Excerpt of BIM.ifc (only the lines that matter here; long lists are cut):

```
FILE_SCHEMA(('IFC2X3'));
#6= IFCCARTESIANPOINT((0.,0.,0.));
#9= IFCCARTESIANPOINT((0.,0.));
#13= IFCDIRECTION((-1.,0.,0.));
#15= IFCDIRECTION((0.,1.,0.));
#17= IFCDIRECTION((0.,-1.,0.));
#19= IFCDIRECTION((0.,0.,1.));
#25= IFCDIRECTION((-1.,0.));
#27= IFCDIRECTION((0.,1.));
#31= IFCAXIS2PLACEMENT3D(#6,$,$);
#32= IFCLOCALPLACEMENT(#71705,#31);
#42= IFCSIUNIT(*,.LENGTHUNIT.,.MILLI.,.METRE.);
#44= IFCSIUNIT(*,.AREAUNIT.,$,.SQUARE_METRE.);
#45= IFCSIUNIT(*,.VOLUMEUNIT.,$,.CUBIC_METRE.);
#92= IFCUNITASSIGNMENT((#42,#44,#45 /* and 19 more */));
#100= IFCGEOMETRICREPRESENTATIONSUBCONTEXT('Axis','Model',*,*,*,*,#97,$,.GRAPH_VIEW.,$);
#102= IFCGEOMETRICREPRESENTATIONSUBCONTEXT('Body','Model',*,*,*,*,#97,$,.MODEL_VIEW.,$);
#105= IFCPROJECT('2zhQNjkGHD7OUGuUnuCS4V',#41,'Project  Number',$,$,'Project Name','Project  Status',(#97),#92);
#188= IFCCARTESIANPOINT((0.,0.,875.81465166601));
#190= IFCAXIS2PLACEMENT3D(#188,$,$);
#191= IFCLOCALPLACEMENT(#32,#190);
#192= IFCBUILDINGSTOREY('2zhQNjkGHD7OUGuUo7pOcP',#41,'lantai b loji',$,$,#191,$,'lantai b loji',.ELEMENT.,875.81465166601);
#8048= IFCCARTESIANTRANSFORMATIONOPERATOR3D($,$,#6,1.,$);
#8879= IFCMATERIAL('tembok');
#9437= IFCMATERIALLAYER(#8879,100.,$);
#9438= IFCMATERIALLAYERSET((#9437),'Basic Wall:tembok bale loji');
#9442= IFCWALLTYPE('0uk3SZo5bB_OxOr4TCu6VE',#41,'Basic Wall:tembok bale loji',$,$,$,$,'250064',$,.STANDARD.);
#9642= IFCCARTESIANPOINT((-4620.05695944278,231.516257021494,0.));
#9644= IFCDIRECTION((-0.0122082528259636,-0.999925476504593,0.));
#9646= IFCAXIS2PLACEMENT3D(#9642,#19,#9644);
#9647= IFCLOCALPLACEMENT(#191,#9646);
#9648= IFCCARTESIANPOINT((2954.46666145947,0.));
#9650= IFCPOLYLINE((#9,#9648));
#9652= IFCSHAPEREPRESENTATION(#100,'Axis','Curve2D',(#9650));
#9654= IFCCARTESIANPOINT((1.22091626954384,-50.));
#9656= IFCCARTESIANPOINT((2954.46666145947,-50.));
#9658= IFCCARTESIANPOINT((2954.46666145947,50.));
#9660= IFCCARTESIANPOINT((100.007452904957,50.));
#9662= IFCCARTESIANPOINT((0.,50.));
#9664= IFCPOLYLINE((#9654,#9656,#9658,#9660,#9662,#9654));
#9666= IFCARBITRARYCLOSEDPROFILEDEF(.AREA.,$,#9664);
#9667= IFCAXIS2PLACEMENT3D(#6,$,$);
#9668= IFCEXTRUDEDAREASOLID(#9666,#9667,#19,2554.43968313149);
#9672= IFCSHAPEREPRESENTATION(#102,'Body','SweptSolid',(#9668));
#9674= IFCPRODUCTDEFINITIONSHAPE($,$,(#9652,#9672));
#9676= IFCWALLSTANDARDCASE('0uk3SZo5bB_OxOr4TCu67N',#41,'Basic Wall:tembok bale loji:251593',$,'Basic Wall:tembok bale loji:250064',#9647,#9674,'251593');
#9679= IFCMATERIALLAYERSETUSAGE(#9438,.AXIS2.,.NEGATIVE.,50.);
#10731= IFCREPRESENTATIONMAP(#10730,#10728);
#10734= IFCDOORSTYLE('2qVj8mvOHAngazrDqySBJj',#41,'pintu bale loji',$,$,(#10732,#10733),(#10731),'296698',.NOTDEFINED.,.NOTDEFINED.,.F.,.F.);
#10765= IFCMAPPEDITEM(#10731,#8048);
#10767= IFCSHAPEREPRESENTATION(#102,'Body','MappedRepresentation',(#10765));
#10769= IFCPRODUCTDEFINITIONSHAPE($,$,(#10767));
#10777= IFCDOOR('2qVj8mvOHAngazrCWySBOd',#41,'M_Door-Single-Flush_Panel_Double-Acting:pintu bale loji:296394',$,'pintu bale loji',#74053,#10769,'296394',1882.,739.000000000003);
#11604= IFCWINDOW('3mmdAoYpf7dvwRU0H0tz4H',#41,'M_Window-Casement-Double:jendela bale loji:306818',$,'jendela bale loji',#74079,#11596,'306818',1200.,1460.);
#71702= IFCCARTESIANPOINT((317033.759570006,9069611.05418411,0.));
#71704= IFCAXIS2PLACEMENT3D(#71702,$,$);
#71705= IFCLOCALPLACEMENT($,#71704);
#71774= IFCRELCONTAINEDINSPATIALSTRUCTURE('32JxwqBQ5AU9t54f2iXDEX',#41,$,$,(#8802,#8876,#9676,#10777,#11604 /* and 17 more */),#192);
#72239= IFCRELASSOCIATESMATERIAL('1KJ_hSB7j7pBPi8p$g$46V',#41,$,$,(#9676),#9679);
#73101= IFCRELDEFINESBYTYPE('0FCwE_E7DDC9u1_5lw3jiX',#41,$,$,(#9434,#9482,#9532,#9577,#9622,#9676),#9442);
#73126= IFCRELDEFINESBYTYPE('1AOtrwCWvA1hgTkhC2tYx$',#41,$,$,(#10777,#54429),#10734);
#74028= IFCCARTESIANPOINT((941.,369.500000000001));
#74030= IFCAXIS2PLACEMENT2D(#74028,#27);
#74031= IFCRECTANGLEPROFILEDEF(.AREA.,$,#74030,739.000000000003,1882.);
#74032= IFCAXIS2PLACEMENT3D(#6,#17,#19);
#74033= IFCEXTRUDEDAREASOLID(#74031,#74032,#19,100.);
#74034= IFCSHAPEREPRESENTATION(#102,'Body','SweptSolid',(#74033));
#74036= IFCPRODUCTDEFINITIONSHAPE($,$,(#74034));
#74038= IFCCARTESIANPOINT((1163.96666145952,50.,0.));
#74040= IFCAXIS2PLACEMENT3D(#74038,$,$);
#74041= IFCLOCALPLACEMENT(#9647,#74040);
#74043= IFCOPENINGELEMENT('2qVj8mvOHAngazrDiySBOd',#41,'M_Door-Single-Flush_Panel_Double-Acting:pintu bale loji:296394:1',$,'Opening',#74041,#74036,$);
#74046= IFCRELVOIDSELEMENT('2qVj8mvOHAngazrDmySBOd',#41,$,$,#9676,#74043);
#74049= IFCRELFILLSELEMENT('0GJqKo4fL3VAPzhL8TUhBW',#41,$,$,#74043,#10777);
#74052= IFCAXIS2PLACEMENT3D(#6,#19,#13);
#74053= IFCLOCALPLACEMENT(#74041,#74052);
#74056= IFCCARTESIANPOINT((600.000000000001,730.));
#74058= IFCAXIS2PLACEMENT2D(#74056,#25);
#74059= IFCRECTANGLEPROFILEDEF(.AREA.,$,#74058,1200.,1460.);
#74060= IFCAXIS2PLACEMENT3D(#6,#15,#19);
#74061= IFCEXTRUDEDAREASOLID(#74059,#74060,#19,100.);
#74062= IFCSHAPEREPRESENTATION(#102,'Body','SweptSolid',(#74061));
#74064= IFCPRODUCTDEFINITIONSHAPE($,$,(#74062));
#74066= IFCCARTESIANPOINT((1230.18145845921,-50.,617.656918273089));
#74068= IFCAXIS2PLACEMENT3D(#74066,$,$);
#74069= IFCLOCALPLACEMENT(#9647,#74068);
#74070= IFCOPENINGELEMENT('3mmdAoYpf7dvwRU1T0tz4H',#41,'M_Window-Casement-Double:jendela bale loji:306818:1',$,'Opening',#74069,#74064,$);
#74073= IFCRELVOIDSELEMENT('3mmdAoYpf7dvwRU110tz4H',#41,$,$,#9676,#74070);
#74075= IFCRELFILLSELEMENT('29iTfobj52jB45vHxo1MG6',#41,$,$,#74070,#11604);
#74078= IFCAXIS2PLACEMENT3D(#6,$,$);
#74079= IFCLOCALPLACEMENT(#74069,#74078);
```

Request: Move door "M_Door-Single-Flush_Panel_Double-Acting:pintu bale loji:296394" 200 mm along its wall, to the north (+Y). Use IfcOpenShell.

```python
import ifcopenshell
import ifcopenshell.api.geometry
import ifcopenshell.util.placement
import ifcopenshell.util.unit

model = ifcopenshell.open("BIM.ifc")
unit_scale = ifcopenshell.util.unit.calculate_unit_scale(model)

door = model.by_guid("2qVj8mvOHAngazrCWySBOd")
opening = door.FillsVoids[0].RelatingOpeningElement
wall = opening.VoidsElements[0].RelatingBuildingElement

wall_matrix = ifcopenshell.util.placement.get_local_placement(wall.ObjectPlacement)
shift = wall_matrix[:3, 0] * -0.2 / unit_scale
before = ifcopenshell.util.placement.get_local_placement(door.ObjectPlacement)[:3, 3].copy()

# The door is placed relative to its opening, so it follows when the opening moves.
matrix = ifcopenshell.util.placement.get_local_placement(opening.ObjectPlacement)
matrix[:3, 3] += shift
ifcopenshell.api.geometry.edit_object_placement(
    model, product=opening, matrix=matrix, is_si=False, should_transform_children=True
)

after = ifcopenshell.util.placement.get_local_placement(door.ObjectPlacement)[:3, 3]
print("door moved by", (after - before).round(3) + 0.0)

model.write("BIM_updated.ifc")
```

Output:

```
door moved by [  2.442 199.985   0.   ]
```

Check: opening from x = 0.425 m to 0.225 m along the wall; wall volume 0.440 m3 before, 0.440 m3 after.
